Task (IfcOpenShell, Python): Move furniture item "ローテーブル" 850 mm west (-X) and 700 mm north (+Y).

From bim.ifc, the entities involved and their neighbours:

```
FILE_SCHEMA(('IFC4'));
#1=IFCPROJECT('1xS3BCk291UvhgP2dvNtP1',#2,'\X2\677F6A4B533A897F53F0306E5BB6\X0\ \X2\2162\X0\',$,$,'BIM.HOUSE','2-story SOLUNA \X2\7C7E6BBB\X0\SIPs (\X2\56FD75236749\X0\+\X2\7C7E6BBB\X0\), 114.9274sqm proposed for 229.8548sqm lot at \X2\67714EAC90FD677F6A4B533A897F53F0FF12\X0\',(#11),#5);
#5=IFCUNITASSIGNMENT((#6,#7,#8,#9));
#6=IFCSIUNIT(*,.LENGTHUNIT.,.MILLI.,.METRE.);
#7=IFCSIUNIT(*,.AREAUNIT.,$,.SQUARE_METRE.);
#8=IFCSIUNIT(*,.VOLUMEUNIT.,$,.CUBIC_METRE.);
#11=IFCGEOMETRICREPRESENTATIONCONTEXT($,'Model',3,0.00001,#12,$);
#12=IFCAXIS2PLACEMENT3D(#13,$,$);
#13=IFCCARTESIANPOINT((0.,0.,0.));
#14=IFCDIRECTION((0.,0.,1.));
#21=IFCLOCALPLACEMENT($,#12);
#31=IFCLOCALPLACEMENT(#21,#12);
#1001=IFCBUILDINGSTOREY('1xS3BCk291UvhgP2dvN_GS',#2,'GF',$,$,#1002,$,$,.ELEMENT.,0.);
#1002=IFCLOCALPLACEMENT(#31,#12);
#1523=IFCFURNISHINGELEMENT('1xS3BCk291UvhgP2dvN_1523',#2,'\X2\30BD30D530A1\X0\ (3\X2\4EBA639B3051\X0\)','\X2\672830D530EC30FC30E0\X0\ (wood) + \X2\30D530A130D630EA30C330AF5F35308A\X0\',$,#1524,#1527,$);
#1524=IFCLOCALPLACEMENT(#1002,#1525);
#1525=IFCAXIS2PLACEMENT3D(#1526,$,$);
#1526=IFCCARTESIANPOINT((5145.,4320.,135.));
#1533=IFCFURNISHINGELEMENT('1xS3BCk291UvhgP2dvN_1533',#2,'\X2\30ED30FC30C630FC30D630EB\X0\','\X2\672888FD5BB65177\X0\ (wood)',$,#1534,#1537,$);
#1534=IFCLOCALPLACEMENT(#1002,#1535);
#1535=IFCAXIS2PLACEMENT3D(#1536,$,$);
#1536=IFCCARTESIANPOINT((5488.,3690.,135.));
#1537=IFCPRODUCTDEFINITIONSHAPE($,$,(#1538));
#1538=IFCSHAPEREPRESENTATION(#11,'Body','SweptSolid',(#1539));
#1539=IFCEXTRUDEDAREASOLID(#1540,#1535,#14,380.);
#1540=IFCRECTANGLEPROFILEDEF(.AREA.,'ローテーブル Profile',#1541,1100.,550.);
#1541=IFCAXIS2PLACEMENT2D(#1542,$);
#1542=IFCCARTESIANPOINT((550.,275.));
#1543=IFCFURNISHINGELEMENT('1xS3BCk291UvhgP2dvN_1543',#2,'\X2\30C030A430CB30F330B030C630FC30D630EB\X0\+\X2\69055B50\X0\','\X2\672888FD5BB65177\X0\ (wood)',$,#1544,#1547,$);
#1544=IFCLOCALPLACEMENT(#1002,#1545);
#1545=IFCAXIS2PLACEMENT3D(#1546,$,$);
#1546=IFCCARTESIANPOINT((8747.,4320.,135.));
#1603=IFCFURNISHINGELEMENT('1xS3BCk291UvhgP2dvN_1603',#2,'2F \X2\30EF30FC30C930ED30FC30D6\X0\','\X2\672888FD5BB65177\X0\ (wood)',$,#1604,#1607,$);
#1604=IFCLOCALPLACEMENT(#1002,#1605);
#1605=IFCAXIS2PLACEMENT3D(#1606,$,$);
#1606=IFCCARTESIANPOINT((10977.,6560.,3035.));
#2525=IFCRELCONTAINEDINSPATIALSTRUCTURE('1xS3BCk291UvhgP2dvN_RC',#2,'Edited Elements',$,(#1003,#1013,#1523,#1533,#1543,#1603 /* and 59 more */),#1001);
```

```python
import ifcopenshell
import ifcopenshell.api.geometry
import ifcopenshell.util.placement
import ifcopenshell.util.unit

model = ifcopenshell.open("bim.ifc")
unit_scale = ifcopenshell.util.unit.calculate_unit_scale(model)

item = model.by_id(1533)
matrix = ifcopenshell.util.placement.get_local_placement(item.ObjectPlacement)
matrix[0, 3] -= 0.85 / unit_scale
matrix[1, 3] += 0.7 / unit_scale
ifcopenshell.api.geometry.edit_object_placement(model, product=item, matrix=matrix, is_si=False)

print(ifcopenshell.util.placement.get_local_placement(item.ObjectPlacement).round(3) + 0.0)

model.write("bim_updated.ifc")
```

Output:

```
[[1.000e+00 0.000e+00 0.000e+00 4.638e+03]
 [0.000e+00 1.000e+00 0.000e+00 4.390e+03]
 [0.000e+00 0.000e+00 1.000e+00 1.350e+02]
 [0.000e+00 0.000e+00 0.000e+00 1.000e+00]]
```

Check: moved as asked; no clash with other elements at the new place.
